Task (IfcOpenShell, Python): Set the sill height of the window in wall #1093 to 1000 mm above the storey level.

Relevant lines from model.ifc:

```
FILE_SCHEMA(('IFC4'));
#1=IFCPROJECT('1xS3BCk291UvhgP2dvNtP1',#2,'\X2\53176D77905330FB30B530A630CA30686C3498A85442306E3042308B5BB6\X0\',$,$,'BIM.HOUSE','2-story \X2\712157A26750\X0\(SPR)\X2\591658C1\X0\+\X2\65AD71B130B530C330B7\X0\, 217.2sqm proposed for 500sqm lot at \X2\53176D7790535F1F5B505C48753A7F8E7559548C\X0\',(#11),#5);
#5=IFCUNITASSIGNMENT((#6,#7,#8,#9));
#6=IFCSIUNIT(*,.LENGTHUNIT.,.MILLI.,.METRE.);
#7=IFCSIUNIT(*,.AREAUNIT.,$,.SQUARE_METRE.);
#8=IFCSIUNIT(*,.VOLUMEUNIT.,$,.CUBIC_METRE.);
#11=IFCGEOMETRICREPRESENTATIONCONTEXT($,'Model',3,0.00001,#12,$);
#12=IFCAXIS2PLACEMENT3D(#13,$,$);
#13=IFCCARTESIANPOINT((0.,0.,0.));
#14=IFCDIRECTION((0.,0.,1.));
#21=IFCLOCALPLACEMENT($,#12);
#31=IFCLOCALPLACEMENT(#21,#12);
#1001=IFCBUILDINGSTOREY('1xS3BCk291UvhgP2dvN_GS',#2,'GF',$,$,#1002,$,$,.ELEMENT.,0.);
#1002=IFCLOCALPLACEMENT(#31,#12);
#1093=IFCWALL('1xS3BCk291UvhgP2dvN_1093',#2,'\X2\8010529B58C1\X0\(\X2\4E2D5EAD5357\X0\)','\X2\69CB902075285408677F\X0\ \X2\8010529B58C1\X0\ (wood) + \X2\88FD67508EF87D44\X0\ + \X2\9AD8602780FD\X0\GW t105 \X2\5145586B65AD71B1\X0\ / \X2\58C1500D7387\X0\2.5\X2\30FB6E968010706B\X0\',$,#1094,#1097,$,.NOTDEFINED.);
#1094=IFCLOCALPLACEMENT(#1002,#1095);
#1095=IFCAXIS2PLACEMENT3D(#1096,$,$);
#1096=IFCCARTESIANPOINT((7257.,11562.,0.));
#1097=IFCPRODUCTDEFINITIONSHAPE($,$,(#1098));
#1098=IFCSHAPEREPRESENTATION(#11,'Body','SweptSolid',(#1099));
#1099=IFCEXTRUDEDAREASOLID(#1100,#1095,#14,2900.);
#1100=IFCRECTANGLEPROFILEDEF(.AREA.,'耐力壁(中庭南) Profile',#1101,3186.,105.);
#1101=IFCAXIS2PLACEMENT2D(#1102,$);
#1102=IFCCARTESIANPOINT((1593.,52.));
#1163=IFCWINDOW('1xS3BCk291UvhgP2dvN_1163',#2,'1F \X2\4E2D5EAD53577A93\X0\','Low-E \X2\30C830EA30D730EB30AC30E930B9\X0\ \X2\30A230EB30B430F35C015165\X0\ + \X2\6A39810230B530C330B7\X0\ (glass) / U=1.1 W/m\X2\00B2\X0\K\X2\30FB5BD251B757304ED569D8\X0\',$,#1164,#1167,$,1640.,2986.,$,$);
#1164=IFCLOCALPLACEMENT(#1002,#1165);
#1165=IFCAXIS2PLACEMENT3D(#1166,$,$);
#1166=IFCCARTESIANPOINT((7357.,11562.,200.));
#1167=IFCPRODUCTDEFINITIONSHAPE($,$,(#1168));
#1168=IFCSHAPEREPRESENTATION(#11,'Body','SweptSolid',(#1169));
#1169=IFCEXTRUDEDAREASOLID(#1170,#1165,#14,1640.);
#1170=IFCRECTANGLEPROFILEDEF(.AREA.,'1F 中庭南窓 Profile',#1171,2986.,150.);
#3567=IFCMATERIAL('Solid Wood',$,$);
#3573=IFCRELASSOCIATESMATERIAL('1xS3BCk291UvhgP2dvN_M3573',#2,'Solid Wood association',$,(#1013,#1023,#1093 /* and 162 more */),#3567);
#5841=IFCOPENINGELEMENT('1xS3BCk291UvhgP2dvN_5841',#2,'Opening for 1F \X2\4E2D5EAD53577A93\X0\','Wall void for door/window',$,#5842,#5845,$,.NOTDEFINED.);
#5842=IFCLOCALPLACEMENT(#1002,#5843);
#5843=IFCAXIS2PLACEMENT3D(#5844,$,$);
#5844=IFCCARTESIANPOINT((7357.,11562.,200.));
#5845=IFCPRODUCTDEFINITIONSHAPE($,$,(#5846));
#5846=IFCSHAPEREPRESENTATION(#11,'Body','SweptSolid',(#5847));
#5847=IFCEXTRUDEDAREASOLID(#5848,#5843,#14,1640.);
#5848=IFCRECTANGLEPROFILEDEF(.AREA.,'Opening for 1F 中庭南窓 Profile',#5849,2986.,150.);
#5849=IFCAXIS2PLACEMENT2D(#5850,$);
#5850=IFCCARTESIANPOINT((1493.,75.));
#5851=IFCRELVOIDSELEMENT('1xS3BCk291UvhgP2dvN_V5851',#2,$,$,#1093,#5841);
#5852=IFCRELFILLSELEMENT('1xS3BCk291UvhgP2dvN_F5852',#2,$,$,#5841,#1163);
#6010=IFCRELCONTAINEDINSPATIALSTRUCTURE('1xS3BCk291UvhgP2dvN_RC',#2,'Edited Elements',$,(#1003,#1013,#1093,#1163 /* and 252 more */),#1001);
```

```python
import numpy as np
import ifcopenshell
import ifcopenshell.api.geometry
import ifcopenshell.geom
import ifcopenshell.util.element
import ifcopenshell.util.placement
import ifcopenshell.util.shape
import ifcopenshell.util.unit

model = ifcopenshell.open("model.ifc")
unit_scale = ifcopenshell.util.unit.calculate_unit_scale(model)

window = model.by_id(1163)
opening = window.FillsVoids[0].RelatingOpeningElement
storey = ifcopenshell.util.element.get_container(window, ifc_class="IfcBuildingStorey")
level = ifcopenshell.util.placement.get_local_placement(storey.ObjectPlacement)[2, 3]

# The opening's origin need not be at the sill, so measure its lowest point.
shape = ifcopenshell.geom.create_shape(ifcopenshell.geom.settings(), opening)
bottom = ifcopenshell.util.shape.get_shape_bottom_elevation(shape, shape.geometry) / unit_scale
dz = level + 1000.0 - bottom

shift = np.array([0.0, 0.0, dz])
# The window is not placed relative to its opening, so move both.
for product in (opening, window):
    matrix = ifcopenshell.util.placement.get_local_placement(product.ObjectPlacement)
    matrix[:3, 3] += shift
    ifcopenshell.api.geometry.edit_object_placement(model, product=product, matrix=matrix, is_si=False)

print(f"moved by {dz * unit_scale:+.3f} m")

model.write("model_rev.ifc")
```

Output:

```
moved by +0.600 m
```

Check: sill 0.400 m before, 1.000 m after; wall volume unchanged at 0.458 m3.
